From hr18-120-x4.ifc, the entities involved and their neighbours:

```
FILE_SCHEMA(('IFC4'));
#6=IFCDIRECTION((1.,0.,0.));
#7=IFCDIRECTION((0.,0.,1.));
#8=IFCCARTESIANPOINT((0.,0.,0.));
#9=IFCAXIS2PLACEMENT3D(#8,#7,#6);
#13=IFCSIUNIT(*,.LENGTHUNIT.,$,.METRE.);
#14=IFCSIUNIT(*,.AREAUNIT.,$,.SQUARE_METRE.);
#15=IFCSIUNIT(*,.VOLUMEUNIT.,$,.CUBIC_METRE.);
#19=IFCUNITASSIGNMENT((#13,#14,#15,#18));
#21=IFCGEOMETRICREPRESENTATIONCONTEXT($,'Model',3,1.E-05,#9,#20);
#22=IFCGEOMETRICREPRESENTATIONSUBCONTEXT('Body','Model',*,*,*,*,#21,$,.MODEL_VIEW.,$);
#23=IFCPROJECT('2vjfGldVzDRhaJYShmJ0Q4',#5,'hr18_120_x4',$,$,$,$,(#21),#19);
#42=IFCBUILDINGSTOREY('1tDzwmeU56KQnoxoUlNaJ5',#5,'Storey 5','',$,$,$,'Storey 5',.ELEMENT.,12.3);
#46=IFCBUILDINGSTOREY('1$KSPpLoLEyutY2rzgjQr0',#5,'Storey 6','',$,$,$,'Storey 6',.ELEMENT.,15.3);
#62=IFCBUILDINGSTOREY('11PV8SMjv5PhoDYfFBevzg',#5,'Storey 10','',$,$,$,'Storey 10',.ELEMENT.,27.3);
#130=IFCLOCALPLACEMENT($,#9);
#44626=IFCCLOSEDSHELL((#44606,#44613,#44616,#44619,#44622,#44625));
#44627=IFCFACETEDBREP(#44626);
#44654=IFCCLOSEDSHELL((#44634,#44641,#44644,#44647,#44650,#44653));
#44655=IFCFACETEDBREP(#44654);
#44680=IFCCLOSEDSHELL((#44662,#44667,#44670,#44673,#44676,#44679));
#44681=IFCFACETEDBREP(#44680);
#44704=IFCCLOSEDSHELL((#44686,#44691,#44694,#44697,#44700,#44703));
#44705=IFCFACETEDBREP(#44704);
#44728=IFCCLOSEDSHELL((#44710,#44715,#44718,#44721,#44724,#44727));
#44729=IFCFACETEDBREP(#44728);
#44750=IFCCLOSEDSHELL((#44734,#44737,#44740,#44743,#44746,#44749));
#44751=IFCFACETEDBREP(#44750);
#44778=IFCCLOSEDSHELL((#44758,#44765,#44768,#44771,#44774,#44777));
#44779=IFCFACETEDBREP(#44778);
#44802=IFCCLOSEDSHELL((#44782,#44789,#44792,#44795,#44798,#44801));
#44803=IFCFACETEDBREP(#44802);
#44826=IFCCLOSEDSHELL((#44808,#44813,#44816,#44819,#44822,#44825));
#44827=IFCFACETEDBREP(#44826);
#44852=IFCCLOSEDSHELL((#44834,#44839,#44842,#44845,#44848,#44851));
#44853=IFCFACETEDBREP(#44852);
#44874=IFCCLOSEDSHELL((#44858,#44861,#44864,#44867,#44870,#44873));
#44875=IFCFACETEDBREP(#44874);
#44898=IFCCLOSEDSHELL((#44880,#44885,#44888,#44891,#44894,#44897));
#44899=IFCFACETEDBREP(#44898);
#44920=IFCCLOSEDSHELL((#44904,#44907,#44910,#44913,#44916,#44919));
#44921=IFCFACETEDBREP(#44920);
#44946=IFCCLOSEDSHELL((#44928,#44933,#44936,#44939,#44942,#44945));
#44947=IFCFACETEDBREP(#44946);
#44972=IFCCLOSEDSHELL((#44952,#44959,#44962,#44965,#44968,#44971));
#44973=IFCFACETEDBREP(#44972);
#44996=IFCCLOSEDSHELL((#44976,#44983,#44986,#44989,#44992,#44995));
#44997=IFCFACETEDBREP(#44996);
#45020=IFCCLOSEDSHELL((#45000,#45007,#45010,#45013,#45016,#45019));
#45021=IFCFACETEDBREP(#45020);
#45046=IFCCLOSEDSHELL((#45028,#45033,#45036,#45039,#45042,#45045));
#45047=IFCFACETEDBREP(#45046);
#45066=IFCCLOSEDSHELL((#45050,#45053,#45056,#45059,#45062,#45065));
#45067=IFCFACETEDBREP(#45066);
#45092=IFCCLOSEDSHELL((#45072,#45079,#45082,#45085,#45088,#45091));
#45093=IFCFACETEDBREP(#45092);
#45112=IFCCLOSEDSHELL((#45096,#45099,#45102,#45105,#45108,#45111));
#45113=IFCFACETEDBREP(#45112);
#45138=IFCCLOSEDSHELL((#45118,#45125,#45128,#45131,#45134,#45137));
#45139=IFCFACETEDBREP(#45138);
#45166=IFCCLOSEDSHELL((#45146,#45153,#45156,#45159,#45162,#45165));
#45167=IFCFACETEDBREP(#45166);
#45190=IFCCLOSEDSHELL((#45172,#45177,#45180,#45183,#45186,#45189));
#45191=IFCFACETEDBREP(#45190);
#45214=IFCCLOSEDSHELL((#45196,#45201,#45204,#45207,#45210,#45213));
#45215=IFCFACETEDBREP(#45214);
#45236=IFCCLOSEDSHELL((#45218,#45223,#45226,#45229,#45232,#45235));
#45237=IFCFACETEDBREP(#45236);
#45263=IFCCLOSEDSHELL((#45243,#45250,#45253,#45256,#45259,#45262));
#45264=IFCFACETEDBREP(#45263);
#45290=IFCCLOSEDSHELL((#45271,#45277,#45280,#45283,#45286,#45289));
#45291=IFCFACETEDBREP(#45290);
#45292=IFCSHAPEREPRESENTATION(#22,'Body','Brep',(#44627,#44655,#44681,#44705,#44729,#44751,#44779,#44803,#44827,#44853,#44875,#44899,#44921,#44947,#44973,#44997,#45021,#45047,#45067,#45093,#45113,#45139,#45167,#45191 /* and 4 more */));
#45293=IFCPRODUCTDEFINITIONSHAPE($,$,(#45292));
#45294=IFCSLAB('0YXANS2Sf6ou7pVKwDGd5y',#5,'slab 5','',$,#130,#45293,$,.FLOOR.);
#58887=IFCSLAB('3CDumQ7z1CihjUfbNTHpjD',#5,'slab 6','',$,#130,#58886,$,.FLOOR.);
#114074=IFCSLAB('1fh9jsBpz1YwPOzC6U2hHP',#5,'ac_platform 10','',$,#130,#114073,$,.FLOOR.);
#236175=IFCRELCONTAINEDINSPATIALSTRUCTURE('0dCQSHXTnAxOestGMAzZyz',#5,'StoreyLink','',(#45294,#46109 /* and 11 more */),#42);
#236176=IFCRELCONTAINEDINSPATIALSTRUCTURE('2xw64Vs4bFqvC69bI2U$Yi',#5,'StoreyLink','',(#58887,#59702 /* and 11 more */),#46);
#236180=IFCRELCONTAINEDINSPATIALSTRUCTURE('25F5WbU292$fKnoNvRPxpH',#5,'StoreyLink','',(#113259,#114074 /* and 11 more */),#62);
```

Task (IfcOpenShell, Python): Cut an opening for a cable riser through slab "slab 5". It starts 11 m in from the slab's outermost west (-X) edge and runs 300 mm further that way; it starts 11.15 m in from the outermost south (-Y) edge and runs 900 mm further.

```python
import numpy as np
import ifcopenshell
import ifcopenshell.api.feature
import ifcopenshell.api.geometry
import ifcopenshell.api.root
import ifcopenshell.geom
import ifcopenshell.util.placement
import ifcopenshell.util.representation
import ifcopenshell.util.shape
import ifcopenshell.util.unit

model = ifcopenshell.open("hr18-120-x4.ifc")
unit_scale = ifcopenshell.util.unit.calculate_unit_scale(model)
settings = ifcopenshell.geom.settings()


def volume(element):
    """Net volume in cubic metres, openings subtracted."""
    shape = ifcopenshell.geom.create_shape(settings, element)
    return ifcopenshell.util.shape.get_volume(shape.geometry)


slab = model.by_id(45294)
before = volume(slab)

# Extent in the slab's own axes, in metres. The edges named are its -X and -Y sides.
slab_shape = ifcopenshell.geom.create_shape(settings, slab)
vertices = ifcopenshell.util.shape.get_vertices(slab_shape.geometry)
x_min, y_min, bottom = vertices.min(axis=0)
top = vertices[:, 2].max()

opening = ifcopenshell.api.root.create_entity(model, ifc_class="IfcOpeningElement", name="Cable riser opening", predefined_type="OPENING")
context = ifcopenshell.util.representation.get_context(model, "Model", "Body", "MODEL_VIEW")
width, depth = 0.3, 0.9
outline = [(0.0, 0.0), (width, 0.0), (width, depth), (0.0, depth), (0.0, 0.0)]
# Overshoot both faces by 50 mm so the cut is clean.
shape = ifcopenshell.api.geometry.add_slab_representation(
    model, context=context, depth=top - bottom + 0.1, polyline=outline
)
ifcopenshell.api.geometry.assign_representation(model, product=opening, representation=shape)

matrix = ifcopenshell.util.placement.get_local_placement(slab.ObjectPlacement)
matrix[:, 3] = matrix @ np.append(np.array([x_min + 11, y_min + 11.15, bottom - 0.05]) / unit_scale, 1.0)
ifcopenshell.api.geometry.edit_object_placement(model, product=opening, matrix=matrix, is_si=False)
ifcopenshell.api.feature.add_feature(model, feature=opening, element=slab)

after = volume(slab)

print(f"slab volume {before:.3f} -> {after:.3f} m3")

model.write("hr18-120-x4_edited.ifc")
```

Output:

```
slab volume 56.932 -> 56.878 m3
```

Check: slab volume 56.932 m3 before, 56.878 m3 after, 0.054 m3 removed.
